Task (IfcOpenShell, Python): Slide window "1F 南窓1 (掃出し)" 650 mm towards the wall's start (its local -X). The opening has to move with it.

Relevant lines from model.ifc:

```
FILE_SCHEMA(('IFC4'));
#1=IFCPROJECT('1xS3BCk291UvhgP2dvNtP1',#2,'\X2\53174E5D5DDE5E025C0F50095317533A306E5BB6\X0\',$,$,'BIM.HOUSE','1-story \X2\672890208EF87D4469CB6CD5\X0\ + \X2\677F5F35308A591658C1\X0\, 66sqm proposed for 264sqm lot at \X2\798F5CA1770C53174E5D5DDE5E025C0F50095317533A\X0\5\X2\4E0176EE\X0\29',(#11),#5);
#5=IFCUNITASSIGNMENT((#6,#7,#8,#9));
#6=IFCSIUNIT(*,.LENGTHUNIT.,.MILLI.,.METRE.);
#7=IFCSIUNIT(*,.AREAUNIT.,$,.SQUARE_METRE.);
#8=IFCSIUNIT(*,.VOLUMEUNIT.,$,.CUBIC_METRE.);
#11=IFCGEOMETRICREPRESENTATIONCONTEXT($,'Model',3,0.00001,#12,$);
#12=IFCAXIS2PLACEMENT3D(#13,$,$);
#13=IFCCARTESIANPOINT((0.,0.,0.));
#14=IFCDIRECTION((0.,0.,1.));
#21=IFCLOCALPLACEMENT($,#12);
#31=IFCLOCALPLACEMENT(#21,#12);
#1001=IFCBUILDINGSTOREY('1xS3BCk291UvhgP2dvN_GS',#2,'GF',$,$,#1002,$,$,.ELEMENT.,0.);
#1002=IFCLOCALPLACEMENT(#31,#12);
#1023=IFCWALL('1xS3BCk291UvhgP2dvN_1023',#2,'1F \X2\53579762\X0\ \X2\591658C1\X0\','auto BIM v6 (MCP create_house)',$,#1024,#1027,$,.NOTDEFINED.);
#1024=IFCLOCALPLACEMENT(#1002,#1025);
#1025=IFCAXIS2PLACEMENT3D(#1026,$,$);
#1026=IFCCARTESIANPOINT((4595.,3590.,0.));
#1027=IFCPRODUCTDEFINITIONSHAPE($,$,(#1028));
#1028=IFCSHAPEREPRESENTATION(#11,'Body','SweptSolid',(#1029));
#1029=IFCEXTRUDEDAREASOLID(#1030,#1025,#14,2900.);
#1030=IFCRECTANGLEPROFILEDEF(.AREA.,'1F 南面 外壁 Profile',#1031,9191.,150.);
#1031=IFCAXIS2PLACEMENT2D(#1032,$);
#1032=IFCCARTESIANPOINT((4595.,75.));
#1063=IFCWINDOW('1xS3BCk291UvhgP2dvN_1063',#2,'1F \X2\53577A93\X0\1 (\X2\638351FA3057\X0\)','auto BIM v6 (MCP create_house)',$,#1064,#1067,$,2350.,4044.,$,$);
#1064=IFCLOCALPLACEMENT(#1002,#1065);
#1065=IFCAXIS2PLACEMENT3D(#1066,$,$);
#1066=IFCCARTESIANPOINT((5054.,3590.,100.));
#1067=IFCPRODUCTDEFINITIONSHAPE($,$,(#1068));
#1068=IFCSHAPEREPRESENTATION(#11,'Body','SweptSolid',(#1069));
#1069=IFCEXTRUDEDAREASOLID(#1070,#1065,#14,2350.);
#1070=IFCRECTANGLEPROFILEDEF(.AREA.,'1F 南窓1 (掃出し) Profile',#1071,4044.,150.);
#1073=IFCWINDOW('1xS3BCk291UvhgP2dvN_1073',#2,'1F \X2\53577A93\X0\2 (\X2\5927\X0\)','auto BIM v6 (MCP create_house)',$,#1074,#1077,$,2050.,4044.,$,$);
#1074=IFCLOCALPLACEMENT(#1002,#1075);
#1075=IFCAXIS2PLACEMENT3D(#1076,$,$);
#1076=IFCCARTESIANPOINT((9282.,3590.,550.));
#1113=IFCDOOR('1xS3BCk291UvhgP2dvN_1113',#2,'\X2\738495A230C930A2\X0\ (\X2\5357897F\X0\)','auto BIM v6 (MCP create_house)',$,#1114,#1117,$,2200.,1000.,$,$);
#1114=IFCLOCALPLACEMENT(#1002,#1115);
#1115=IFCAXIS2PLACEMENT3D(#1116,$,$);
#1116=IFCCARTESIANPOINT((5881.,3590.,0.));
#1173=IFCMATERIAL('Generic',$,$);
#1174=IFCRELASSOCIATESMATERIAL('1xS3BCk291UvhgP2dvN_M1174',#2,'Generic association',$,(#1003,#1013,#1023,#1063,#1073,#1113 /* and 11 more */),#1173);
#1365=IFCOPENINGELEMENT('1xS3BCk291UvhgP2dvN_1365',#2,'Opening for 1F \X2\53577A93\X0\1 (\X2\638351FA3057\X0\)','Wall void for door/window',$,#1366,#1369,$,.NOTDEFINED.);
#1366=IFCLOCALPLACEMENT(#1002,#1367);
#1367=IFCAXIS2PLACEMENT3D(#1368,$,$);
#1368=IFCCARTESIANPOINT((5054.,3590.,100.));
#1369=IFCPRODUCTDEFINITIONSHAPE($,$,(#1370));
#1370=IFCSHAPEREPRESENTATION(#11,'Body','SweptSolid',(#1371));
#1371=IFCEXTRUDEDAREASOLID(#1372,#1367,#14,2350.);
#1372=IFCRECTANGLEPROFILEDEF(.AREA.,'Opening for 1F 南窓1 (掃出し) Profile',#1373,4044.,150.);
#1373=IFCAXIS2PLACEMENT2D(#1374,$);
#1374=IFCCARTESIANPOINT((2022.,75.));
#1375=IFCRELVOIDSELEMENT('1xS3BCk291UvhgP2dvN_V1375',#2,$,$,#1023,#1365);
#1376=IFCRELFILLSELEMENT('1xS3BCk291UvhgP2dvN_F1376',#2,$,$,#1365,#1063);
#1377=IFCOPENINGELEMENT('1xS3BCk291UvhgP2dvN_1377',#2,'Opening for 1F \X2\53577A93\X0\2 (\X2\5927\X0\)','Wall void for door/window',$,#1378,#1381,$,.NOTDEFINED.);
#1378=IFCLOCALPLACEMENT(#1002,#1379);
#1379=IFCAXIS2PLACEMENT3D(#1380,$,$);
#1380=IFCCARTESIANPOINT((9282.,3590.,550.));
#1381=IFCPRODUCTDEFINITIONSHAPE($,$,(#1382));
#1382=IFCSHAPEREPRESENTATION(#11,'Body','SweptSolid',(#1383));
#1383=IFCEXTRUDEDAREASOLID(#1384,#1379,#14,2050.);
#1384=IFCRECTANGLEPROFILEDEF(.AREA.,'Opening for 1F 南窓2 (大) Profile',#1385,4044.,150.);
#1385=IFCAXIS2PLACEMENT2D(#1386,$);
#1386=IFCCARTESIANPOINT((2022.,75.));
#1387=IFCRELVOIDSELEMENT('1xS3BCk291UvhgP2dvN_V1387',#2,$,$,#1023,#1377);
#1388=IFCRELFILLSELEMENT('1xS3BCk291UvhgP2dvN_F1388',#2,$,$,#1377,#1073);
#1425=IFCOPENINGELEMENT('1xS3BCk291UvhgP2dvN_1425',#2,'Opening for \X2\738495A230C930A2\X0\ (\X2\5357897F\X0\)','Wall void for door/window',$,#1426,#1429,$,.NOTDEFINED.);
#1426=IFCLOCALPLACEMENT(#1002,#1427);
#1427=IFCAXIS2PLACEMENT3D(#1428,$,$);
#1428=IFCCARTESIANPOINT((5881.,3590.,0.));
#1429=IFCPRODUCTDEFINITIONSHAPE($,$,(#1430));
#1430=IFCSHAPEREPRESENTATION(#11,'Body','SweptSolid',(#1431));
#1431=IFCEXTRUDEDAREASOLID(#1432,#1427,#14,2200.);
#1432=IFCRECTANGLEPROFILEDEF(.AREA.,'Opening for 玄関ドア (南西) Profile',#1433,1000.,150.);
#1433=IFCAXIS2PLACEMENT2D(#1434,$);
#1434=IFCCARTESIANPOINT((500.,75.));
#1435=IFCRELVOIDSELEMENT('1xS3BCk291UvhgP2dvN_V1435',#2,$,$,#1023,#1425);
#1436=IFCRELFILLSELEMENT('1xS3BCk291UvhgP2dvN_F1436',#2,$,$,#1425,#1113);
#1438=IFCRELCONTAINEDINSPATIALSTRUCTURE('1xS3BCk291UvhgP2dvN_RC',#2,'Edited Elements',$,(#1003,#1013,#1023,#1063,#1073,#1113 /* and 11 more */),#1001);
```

```python
import ifcopenshell
import ifcopenshell.api.geometry
import ifcopenshell.util.placement
import ifcopenshell.util.unit

model = ifcopenshell.open("model.ifc")
unit_scale = ifcopenshell.util.unit.calculate_unit_scale(model)

window = model.by_guid("1xS3BCk291UvhgP2dvN_1063")
opening = window.FillsVoids[0].RelatingOpeningElement
wall = opening.VoidsElements[0].RelatingBuildingElement

wall_matrix = ifcopenshell.util.placement.get_local_placement(wall.ObjectPlacement)
shift = wall_matrix[:3, 0] * -0.65 / unit_scale
before = ifcopenshell.util.placement.get_local_placement(window.ObjectPlacement)[:3, 3].copy()

# The window is not placed relative to its opening, so move both.
for product in (opening, window):
    matrix = ifcopenshell.util.placement.get_local_placement(product.ObjectPlacement)
    matrix[:3, 3] += shift
    ifcopenshell.api.geometry.edit_object_placement(model, product=product, matrix=matrix, is_si=False)

after = ifcopenshell.util.placement.get_local_placement(window.ObjectPlacement)[:3, 3]
print("window moved by", (after - before).round(3) + 0.0)

model.write("model_rev.ifc")
```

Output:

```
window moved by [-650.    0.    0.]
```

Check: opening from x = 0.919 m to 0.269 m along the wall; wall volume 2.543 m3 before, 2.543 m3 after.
